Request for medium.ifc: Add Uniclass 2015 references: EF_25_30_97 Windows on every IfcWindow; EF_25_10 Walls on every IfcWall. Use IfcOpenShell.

First a look at what the model holds.

```python
import ifcopenshell

model = ifcopenshell.open("medium.ifc")
print(model.schema)
print("classifications:", [c.Name for c in model.by_type("IfcClassification")])
for ifc_class in ("IfcDoor", "IfcRoof", "IfcStair", "IfcWall", "IfcWindow"):
    print(ifc_class, len(model.by_type(ifc_class)))
```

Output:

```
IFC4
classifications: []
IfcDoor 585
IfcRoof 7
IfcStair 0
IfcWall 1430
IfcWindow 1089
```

```python
import ifcopenshell
import ifcopenshell.api.classification

model = ifcopenshell.open("medium.ifc")

system = ifcopenshell.api.classification.add_classification(model, classification="Uniclass 2015")

codes = {
    "IfcWindow": ("EF_25_30_97", "Windows"),
    "IfcWall": ("EF_25_10", "Walls"),
}
for ifc_class, (code, name) in codes.items():
    products = model.by_type(ifc_class)
    ifcopenshell.api.classification.add_reference(
        model, products=products, classification=system, identification=code, name=name
    )
    print(code, len(products))

model.write("medium-out.ifc")
```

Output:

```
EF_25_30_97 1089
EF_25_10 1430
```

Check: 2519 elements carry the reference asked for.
